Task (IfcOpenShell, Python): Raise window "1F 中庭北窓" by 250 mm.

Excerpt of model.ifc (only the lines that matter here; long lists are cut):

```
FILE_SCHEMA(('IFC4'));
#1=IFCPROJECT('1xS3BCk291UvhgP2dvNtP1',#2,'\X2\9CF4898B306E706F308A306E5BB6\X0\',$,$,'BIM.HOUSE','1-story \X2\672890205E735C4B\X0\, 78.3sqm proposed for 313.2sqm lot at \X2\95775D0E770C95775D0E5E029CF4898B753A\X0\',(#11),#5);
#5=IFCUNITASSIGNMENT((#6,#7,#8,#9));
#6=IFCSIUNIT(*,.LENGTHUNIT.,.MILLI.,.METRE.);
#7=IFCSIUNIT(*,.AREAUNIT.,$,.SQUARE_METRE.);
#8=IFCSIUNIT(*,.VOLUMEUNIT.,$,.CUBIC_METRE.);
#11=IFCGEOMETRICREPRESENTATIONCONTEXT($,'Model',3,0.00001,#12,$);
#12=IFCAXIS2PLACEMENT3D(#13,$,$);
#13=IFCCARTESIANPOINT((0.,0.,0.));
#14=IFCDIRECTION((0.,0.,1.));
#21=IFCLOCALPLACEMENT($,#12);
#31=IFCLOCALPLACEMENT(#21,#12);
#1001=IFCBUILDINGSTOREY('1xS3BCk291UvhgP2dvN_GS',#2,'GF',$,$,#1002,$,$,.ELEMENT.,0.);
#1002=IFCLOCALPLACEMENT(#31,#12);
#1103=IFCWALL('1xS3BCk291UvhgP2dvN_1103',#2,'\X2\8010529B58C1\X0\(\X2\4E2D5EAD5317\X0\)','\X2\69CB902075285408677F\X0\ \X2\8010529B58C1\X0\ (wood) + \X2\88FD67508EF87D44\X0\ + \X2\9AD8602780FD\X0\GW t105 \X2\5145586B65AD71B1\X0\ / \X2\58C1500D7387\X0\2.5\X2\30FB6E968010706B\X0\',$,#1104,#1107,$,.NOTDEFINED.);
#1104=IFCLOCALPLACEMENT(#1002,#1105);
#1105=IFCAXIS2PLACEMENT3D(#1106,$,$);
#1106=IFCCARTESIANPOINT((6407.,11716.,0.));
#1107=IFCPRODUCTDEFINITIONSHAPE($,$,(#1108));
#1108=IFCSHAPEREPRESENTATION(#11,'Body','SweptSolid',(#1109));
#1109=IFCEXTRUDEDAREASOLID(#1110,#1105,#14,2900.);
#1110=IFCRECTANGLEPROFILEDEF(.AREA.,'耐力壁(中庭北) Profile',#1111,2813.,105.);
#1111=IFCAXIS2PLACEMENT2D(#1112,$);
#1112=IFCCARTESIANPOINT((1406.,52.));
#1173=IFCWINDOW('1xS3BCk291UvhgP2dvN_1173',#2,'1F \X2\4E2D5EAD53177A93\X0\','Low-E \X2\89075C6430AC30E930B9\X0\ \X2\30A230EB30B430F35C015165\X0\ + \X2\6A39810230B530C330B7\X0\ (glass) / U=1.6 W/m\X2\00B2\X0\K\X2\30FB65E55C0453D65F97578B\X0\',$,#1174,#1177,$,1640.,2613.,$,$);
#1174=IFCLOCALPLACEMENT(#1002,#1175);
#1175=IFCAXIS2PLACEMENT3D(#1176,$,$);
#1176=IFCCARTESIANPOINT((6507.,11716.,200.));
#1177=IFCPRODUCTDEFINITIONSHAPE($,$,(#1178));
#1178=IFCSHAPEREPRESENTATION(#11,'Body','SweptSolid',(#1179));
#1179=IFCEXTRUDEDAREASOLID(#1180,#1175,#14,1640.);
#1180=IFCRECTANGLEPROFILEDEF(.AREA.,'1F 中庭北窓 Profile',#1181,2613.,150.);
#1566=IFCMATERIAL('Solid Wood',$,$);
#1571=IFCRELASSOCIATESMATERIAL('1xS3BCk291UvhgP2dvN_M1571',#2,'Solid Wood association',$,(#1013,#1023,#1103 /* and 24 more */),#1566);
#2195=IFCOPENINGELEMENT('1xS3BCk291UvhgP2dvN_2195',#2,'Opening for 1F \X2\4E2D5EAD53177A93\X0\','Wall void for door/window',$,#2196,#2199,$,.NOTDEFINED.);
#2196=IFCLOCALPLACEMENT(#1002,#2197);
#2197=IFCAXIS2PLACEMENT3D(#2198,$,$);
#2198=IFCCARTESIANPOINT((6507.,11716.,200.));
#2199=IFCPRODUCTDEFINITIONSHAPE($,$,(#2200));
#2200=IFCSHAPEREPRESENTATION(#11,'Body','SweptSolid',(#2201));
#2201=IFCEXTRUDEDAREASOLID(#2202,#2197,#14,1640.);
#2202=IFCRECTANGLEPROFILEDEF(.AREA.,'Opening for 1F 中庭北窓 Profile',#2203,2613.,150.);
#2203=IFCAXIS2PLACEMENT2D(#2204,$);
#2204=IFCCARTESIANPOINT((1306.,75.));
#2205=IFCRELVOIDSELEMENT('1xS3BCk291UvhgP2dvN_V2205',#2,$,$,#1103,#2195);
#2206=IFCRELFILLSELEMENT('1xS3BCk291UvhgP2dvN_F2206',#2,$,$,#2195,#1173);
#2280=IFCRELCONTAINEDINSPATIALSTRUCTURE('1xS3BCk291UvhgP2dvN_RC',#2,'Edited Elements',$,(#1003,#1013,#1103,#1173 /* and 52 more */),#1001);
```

```python
import numpy as np
import ifcopenshell
import ifcopenshell.api.geometry
import ifcopenshell.util.placement
import ifcopenshell.util.unit

model = ifcopenshell.open("model.ifc")
unit_scale = ifcopenshell.util.unit.calculate_unit_scale(model)

window = model.by_guid("1xS3BCk291UvhgP2dvN_1173")
opening = window.FillsVoids[0].RelatingOpeningElement
dz = 0.25 / unit_scale

shift = np.array([0.0, 0.0, dz])
# The window is not placed relative to its opening, so move both.
for product in (opening, window):
    matrix = ifcopenshell.util.placement.get_local_placement(product.ObjectPlacement)
    matrix[:3, 3] += shift
    ifcopenshell.api.geometry.edit_object_placement(model, product=product, matrix=matrix, is_si=False)

print(f"moved by {dz * unit_scale:+.3f} m")

model.write("model_updated.ifc")
```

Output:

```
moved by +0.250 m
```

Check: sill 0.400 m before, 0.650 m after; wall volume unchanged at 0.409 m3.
